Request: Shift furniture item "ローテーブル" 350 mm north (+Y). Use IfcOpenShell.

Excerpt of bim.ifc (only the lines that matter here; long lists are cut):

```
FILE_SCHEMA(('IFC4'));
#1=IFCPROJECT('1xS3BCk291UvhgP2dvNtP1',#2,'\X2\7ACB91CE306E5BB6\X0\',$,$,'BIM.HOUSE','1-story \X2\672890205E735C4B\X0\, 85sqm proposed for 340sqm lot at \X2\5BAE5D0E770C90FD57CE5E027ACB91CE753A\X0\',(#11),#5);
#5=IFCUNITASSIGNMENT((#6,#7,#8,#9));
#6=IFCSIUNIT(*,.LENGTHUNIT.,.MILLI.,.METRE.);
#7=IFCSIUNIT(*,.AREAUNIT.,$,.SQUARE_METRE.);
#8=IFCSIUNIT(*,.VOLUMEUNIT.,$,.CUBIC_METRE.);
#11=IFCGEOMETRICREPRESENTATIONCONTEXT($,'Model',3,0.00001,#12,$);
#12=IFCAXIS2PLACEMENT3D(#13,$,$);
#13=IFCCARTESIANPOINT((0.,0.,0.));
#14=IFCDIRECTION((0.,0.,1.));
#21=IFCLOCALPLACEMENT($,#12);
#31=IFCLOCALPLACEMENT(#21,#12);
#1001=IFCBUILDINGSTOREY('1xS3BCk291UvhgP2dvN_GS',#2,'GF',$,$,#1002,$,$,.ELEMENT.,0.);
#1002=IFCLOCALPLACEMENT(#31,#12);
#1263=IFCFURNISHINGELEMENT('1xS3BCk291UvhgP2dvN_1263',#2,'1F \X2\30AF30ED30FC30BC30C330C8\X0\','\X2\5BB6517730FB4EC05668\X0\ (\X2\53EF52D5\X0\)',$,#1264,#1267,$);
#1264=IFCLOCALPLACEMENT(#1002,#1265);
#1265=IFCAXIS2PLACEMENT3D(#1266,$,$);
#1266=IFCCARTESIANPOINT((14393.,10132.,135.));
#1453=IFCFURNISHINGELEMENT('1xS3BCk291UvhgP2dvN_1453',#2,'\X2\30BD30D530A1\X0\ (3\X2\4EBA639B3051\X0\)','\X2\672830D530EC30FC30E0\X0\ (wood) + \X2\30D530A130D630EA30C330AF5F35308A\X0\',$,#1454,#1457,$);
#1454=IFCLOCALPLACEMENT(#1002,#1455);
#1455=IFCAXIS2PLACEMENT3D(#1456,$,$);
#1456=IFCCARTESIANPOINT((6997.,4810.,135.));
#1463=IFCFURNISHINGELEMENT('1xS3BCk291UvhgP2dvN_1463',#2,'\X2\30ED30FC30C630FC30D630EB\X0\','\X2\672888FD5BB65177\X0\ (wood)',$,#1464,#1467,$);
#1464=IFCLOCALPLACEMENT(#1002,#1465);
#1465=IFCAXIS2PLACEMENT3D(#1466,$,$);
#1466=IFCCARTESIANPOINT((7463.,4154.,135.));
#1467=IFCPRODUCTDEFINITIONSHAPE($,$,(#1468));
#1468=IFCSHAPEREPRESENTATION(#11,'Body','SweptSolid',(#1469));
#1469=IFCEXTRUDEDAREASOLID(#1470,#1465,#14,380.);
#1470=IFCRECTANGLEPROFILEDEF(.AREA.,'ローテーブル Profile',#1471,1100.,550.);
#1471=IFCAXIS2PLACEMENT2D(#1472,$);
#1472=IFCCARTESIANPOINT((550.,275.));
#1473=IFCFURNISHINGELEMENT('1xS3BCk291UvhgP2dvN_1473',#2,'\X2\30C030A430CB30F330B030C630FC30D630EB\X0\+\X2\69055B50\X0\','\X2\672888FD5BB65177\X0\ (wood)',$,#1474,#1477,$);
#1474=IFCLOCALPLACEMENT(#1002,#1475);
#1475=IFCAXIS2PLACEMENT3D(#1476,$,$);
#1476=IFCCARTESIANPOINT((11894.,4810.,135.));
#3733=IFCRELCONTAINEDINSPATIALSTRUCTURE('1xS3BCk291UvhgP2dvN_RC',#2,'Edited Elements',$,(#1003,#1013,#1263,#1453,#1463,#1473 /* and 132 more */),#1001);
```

```python
import ifcopenshell
import ifcopenshell.api.geometry
import ifcopenshell.util.placement

model = ifcopenshell.open("bim.ifc")

item = model.by_guid("1xS3BCk291UvhgP2dvN_1463")
matrix = ifcopenshell.util.placement.get_local_placement(item.ObjectPlacement)
matrix[1, 3] += 350.0
ifcopenshell.api.geometry.edit_object_placement(model, product=item, matrix=matrix, is_si=False)

print(ifcopenshell.util.placement.get_local_placement(item.ObjectPlacement).round(3) + 0.0)

model.write("bim_v2.ifc")
```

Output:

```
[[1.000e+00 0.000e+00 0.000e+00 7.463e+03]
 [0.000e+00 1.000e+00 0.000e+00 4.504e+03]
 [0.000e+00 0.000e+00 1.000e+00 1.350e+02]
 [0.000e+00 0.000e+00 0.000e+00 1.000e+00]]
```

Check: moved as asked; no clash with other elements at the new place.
